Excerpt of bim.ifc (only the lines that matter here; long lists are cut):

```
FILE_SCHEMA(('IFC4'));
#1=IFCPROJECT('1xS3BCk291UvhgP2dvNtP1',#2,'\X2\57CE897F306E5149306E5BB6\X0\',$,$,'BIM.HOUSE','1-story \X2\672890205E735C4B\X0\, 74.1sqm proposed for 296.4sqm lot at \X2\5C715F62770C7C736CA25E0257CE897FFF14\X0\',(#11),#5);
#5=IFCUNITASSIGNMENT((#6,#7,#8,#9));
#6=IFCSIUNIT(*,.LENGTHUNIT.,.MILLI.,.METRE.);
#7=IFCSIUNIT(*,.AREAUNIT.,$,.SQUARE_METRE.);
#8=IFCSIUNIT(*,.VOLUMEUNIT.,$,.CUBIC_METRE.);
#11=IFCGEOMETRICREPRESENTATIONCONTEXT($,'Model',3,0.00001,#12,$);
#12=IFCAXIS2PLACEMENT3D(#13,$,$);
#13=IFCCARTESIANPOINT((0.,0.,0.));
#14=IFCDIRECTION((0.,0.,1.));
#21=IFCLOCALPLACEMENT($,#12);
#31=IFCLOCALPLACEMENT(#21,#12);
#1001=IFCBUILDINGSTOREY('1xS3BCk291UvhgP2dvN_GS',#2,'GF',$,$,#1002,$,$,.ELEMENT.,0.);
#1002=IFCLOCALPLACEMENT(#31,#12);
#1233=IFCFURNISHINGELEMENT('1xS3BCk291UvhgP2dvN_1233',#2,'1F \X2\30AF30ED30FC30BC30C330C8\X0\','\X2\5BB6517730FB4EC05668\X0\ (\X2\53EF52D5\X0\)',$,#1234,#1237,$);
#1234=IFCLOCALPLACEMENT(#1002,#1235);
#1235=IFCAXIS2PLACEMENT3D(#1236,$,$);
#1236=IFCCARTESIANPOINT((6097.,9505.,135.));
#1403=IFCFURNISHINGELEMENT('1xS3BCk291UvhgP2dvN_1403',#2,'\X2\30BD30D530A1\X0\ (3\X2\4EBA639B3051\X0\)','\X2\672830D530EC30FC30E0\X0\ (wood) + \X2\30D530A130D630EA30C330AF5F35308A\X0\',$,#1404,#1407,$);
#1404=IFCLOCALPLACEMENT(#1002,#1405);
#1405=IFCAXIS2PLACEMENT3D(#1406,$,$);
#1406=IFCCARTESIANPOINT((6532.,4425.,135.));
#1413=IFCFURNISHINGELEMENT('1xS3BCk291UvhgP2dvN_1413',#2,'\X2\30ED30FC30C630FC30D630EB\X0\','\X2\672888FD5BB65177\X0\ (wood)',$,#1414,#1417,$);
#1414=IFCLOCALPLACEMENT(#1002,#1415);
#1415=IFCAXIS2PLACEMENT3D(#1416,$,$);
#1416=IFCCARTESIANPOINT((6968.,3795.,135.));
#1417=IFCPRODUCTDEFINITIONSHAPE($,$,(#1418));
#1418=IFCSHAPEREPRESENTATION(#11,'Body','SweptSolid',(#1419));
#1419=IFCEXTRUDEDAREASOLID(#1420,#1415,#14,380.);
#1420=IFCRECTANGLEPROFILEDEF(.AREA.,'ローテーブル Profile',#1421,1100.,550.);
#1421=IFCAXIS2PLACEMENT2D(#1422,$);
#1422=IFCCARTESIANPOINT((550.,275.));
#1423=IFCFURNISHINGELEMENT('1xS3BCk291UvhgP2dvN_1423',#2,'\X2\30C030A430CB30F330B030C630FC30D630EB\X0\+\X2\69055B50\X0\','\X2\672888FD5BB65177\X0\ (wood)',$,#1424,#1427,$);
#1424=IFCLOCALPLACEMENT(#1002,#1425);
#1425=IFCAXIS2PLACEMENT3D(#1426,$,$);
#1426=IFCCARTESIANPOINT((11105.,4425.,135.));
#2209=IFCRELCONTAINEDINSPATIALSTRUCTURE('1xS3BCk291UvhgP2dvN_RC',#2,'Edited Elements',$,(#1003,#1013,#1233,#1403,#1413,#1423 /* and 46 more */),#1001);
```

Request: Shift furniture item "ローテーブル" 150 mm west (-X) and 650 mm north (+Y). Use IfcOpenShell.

```python
import ifcopenshell
import ifcopenshell.api.geometry
import ifcopenshell.util.placement
import ifcopenshell.util.unit

model = ifcopenshell.open("bim.ifc")
unit_scale = ifcopenshell.util.unit.calculate_unit_scale(model)

item = model.by_guid("1xS3BCk291UvhgP2dvN_1413")
matrix = ifcopenshell.util.placement.get_local_placement(item.ObjectPlacement)
matrix[0, 3] -= 0.15 / unit_scale
matrix[1, 3] += 0.65 / unit_scale
ifcopenshell.api.geometry.edit_object_placement(model, product=item, matrix=matrix, is_si=False)

print(ifcopenshell.util.placement.get_local_placement(item.ObjectPlacement).round(3) + 0.0)

model.write("bim_updated.ifc")
```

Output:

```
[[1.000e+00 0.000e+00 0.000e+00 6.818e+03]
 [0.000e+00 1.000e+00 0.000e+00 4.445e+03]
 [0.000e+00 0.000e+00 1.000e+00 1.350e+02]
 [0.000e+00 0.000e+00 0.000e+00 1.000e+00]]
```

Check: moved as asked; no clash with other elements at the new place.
